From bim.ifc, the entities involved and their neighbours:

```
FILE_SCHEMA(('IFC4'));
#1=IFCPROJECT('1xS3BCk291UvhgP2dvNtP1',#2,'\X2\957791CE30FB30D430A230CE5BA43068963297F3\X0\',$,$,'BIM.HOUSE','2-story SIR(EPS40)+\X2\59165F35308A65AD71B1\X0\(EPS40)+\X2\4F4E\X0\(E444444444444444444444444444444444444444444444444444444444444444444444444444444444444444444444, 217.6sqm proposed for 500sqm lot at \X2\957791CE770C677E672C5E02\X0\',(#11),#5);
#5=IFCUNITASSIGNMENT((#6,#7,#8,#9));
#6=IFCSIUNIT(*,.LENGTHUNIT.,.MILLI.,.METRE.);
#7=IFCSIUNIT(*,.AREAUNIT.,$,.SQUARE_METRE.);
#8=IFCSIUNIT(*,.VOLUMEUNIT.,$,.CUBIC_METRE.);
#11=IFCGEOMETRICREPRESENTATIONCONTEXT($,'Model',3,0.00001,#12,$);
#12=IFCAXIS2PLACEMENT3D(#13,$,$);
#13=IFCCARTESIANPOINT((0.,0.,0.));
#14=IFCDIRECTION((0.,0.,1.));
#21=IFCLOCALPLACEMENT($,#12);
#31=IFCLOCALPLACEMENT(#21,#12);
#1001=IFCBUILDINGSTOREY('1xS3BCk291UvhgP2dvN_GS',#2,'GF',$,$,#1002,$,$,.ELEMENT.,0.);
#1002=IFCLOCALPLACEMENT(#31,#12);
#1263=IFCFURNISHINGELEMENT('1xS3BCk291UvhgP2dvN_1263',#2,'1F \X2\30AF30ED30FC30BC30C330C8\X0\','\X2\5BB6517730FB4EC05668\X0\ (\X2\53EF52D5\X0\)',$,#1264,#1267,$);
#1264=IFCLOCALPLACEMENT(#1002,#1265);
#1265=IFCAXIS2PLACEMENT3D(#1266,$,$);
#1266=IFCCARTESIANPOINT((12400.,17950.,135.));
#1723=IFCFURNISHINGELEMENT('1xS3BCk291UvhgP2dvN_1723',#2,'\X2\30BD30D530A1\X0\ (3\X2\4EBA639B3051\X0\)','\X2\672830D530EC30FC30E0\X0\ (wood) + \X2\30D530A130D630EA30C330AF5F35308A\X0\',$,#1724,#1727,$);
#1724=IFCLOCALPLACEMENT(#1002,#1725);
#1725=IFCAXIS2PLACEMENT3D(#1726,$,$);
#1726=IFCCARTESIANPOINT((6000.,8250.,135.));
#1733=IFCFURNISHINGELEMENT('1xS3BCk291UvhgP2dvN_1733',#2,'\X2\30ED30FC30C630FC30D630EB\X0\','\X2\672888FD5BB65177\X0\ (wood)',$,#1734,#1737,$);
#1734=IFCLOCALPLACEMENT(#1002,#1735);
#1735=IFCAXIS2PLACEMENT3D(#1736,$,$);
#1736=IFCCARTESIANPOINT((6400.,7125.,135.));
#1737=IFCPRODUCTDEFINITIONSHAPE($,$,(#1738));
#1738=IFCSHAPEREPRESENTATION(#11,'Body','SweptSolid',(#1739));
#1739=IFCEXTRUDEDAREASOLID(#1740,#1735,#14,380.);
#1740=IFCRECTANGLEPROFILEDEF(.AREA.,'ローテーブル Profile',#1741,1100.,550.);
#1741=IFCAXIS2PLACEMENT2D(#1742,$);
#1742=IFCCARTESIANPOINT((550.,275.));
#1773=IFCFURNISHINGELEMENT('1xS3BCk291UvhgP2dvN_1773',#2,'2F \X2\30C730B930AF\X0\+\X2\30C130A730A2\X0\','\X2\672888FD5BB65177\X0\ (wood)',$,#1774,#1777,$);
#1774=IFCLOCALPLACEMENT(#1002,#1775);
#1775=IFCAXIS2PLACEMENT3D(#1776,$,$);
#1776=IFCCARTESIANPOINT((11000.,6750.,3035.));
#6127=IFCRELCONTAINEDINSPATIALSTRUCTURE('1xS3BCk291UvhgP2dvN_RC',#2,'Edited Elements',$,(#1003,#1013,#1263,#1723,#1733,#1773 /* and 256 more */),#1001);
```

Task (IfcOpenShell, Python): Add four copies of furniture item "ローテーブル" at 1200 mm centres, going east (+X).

```python
import numpy as np
import ifcopenshell
import ifcopenshell.api.geometry
import ifcopenshell.api.root
import ifcopenshell.util.element
import ifcopenshell.util.placement
import ifcopenshell.util.unit

model = ifcopenshell.open("bim.ifc")
unit_scale = ifcopenshell.util.unit.calculate_unit_scale(model)


def reuse_history(source, copy):
    """copy_class also copies each property set's owner history, people and application; keep the originals."""
    for rel in copy.IsDefinedBy:
        if rel.is_a("IfcRelDefinesByProperties") and (history := rel.RelatingPropertyDefinition.OwnerHistory):
            rel.RelatingPropertyDefinition.OwnerHistory = source.OwnerHistory
            ifcopenshell.util.element.remove_deep2(model, history)


source = model.by_guid("1xS3BCk291UvhgP2dvN_1733")
base = ifcopenshell.util.placement.get_local_placement(source.ObjectPlacement)
step = np.array([1.0, 0.0, 0.0]) * 1.2 / unit_scale

for i in range(1, 5):
    copy = ifcopenshell.api.root.copy_class(model, product=source)
    copy.Representation = ifcopenshell.util.element.copy_deep(
        model, source.Representation, exclude=["IfcGeometricRepresentationContext", "IfcRepresentationMap"]
    )
    reuse_history(source, copy)
    matrix = base.copy()
    matrix[:3, 3] += i * step
    print("added at", matrix[:3, 3].round(3) + 0.0)
    ifcopenshell.api.geometry.edit_object_placement(model, product=copy, matrix=matrix, is_si=False)

model.write("bim_v2.ifc")
```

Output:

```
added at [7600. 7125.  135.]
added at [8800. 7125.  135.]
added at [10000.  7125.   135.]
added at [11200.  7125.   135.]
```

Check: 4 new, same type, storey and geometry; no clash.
